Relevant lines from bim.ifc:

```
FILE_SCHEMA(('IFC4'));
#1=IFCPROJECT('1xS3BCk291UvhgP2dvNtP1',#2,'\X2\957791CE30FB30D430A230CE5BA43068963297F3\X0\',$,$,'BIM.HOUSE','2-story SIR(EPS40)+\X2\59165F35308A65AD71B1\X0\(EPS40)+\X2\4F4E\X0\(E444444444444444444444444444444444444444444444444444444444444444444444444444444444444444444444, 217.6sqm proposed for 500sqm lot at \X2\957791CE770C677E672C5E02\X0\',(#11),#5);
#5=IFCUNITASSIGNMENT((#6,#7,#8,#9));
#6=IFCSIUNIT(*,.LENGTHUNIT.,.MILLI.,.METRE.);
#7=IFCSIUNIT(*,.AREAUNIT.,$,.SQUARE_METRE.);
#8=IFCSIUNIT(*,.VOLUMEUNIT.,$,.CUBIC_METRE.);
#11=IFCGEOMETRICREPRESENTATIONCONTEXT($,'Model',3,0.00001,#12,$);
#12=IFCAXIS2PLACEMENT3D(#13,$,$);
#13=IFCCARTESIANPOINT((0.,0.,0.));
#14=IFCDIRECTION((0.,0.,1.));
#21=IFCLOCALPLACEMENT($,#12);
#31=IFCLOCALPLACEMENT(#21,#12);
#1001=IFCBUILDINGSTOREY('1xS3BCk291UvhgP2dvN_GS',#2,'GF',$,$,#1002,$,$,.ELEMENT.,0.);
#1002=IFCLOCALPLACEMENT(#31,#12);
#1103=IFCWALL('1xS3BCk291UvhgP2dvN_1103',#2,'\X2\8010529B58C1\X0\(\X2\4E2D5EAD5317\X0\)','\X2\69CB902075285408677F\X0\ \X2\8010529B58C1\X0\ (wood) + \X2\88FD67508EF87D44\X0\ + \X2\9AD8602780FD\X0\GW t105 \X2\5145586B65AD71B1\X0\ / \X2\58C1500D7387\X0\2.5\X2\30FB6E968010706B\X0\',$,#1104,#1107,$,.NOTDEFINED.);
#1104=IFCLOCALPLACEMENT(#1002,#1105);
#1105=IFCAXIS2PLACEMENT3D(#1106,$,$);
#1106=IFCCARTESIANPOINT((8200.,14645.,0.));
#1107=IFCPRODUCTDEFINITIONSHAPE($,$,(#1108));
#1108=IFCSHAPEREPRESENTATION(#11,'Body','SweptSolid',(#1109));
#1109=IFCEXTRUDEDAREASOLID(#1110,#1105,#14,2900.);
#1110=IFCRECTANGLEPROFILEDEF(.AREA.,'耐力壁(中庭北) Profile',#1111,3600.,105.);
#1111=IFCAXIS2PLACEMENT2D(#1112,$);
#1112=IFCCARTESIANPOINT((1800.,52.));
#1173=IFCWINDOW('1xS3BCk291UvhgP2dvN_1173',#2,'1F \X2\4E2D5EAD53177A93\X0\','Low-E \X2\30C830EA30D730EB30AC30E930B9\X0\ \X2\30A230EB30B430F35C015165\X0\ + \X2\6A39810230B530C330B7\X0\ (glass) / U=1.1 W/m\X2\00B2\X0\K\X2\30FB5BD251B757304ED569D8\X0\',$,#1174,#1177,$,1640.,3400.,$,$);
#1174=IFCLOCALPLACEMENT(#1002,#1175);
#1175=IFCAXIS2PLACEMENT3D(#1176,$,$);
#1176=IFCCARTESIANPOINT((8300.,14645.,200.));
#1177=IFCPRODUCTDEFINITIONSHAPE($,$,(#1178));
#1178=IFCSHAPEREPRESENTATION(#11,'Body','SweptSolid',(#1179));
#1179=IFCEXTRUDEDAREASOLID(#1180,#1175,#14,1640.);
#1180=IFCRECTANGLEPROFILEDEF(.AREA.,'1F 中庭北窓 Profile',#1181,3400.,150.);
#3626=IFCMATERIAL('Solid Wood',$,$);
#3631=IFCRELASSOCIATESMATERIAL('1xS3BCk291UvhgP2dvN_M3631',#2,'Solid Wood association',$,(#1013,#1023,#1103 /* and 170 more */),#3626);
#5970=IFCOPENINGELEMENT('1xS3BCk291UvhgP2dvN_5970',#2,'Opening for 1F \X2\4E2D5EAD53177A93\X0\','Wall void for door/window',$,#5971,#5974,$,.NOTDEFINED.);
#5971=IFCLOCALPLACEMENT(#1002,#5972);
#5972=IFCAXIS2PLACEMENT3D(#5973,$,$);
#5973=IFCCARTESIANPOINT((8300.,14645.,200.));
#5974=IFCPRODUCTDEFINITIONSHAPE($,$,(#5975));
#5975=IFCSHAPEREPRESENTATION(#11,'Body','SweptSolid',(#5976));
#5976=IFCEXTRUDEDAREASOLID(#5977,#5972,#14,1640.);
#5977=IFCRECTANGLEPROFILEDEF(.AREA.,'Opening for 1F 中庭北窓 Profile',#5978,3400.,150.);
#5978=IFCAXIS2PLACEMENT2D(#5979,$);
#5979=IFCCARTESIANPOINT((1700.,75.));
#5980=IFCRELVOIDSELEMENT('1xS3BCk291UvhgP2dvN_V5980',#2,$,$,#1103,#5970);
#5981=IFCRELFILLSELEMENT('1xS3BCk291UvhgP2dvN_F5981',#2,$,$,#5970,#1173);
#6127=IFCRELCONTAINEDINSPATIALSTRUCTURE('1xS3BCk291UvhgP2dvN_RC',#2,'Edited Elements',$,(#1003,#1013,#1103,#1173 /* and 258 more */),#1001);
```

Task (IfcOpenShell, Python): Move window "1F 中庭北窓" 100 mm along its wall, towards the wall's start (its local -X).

```python
import ifcopenshell
import ifcopenshell.api.geometry
import ifcopenshell.util.placement
import ifcopenshell.util.unit

model = ifcopenshell.open("bim.ifc")
unit_scale = ifcopenshell.util.unit.calculate_unit_scale(model)

window = model.by_id(1173)
opening = window.FillsVoids[0].RelatingOpeningElement
wall = opening.VoidsElements[0].RelatingBuildingElement

wall_matrix = ifcopenshell.util.placement.get_local_placement(wall.ObjectPlacement)
shift = wall_matrix[:3, 0] * -0.1 / unit_scale
before = ifcopenshell.util.placement.get_local_placement(window.ObjectPlacement)[:3, 3].copy()

# The window is not placed relative to its opening, so move both.
for product in (opening, window):
    matrix = ifcopenshell.util.placement.get_local_placement(product.ObjectPlacement)
    matrix[:3, 3] += shift
    ifcopenshell.api.geometry.edit_object_placement(model, product=product, matrix=matrix, is_si=False)

after = ifcopenshell.util.placement.get_local_placement(window.ObjectPlacement)[:3, 3]
print("window moved by", (after - before).round(3) + 0.0)

model.write("bim_updated.ifc")
```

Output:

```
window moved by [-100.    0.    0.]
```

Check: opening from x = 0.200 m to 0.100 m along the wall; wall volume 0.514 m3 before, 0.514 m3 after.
